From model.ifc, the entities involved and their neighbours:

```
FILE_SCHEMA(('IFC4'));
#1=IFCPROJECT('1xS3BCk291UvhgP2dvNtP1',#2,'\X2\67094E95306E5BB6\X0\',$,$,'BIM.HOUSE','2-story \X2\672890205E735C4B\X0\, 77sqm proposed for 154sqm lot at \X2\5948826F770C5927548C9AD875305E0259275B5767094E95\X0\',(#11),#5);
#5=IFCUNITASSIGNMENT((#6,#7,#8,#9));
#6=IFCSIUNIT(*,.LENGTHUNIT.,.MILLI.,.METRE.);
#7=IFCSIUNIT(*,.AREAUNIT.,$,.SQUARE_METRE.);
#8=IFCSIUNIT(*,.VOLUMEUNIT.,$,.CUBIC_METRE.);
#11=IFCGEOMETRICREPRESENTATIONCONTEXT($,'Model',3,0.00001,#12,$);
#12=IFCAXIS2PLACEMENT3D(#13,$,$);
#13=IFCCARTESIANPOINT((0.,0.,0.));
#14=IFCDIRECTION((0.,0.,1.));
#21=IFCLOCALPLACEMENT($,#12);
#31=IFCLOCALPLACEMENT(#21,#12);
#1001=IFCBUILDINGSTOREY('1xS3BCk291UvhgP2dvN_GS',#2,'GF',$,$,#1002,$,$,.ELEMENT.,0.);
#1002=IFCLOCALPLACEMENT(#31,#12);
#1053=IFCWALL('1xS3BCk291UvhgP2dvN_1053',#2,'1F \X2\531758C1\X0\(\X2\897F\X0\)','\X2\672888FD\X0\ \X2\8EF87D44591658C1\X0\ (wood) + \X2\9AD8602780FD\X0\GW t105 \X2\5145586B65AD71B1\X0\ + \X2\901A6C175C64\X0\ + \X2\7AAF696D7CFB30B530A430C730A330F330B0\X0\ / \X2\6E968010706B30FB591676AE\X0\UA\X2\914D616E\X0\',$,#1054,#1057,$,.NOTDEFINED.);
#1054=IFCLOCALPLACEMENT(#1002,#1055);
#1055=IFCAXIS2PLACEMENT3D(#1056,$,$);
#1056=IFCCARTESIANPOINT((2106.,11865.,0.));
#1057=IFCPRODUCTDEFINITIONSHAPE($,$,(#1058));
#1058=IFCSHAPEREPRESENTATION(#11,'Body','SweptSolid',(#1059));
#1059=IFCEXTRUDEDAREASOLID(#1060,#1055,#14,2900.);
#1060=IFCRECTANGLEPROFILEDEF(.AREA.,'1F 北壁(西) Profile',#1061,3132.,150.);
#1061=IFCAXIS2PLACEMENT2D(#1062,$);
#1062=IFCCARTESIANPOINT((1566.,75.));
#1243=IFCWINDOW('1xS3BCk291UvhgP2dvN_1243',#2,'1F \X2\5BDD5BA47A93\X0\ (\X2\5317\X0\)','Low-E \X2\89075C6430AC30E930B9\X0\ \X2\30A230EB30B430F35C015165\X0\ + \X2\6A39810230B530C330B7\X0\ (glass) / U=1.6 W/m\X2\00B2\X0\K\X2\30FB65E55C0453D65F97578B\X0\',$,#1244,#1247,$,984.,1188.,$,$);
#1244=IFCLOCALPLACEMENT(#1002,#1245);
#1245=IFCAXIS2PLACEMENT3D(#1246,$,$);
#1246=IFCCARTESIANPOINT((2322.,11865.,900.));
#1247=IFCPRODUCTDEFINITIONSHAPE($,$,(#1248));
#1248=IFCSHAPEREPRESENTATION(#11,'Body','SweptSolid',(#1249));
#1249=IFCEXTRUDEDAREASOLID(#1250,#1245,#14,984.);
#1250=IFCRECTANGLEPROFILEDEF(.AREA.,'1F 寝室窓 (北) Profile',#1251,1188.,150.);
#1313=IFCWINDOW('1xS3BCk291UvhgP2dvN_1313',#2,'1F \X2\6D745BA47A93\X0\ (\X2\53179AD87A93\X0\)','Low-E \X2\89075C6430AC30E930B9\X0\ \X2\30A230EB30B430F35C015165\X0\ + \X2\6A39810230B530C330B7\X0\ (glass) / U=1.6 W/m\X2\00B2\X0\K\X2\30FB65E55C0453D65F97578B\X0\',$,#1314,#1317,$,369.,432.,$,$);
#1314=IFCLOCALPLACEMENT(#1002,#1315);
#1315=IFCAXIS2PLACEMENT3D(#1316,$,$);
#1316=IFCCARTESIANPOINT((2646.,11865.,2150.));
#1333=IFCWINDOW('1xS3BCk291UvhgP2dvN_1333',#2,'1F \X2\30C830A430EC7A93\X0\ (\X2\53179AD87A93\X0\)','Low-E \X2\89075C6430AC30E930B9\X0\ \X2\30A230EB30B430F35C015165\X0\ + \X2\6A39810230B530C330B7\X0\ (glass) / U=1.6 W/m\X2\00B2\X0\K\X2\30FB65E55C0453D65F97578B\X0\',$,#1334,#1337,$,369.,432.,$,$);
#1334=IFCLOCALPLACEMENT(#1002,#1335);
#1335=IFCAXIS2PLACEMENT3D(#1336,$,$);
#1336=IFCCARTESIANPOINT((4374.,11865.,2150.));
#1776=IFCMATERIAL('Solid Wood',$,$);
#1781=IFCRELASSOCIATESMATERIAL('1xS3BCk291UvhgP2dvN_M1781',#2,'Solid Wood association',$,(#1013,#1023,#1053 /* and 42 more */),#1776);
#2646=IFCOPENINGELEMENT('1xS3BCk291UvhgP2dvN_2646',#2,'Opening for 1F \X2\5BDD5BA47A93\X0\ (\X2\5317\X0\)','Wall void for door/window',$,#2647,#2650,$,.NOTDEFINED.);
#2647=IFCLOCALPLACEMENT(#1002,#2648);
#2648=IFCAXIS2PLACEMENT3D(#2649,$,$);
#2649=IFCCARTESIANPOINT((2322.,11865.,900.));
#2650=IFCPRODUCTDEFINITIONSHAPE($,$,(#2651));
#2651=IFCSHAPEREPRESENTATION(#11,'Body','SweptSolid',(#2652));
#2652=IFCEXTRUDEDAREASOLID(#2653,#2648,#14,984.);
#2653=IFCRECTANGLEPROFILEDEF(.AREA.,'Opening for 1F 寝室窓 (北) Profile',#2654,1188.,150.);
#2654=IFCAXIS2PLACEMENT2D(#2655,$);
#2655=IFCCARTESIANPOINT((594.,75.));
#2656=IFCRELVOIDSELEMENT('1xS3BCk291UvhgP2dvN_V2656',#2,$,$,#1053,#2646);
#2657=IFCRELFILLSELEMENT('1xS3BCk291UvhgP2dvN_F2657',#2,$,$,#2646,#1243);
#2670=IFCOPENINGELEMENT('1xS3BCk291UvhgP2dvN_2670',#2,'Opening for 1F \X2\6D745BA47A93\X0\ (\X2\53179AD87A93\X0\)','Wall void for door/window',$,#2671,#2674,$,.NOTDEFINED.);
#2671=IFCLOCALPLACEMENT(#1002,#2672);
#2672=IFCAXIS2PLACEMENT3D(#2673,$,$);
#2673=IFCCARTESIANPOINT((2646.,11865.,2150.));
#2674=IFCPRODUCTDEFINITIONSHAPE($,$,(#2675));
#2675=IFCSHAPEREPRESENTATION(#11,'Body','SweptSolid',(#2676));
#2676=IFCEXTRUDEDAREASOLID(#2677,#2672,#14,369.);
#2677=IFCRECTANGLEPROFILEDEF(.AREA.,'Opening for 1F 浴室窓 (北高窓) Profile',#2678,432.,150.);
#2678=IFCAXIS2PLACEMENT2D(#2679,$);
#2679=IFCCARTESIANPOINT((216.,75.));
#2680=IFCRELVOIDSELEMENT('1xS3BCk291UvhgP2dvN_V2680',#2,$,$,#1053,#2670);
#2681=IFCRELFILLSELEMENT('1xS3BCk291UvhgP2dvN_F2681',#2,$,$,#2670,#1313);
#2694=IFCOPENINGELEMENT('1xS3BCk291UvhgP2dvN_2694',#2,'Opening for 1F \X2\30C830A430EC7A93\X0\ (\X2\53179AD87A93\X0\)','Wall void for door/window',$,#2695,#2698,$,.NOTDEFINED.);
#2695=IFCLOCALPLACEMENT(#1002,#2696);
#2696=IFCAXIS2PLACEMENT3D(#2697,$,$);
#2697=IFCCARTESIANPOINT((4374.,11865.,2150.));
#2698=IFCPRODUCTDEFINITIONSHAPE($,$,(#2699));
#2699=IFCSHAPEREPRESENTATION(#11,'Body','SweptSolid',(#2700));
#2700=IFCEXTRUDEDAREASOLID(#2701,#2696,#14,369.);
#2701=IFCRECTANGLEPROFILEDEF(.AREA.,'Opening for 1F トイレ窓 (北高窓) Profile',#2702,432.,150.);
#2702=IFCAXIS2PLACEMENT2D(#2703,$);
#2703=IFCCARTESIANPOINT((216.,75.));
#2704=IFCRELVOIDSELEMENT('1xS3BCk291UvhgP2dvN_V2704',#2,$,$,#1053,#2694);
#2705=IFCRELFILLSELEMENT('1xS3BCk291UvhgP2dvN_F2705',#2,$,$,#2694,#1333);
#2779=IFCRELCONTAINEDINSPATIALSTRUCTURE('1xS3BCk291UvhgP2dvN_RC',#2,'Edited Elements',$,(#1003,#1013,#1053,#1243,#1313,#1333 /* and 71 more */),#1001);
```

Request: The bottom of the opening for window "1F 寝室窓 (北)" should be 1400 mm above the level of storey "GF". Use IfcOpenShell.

```python
import numpy as np
import ifcopenshell
import ifcopenshell.api.geometry
import ifcopenshell.geom
import ifcopenshell.util.element
import ifcopenshell.util.placement
import ifcopenshell.util.shape
import ifcopenshell.util.unit

model = ifcopenshell.open("model.ifc")
unit_scale = ifcopenshell.util.unit.calculate_unit_scale(model)

window = model.by_guid("1xS3BCk291UvhgP2dvN_1243")
opening = window.FillsVoids[0].RelatingOpeningElement
storey = ifcopenshell.util.element.get_container(window, ifc_class="IfcBuildingStorey")
level = ifcopenshell.util.placement.get_local_placement(storey.ObjectPlacement)[2, 3]

# The opening's origin need not be at the sill, so measure its lowest point.
shape = ifcopenshell.geom.create_shape(ifcopenshell.geom.settings(), opening)
bottom = ifcopenshell.util.shape.get_shape_bottom_elevation(shape, shape.geometry) / unit_scale
dz = level + 1400.0 - bottom

shift = np.array([0.0, 0.0, dz])
# The window is not placed relative to its opening, so move both.
for product in (opening, window):
    matrix = ifcopenshell.util.placement.get_local_placement(product.ObjectPlacement)
    matrix[:3, 3] += shift
    ifcopenshell.api.geometry.edit_object_placement(model, product=product, matrix=matrix, is_si=False)

print(f"moved by {dz * unit_scale:+.3f} m")

model.write("model_edited.ifc")
```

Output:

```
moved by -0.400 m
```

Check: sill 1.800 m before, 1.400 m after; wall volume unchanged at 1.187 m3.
